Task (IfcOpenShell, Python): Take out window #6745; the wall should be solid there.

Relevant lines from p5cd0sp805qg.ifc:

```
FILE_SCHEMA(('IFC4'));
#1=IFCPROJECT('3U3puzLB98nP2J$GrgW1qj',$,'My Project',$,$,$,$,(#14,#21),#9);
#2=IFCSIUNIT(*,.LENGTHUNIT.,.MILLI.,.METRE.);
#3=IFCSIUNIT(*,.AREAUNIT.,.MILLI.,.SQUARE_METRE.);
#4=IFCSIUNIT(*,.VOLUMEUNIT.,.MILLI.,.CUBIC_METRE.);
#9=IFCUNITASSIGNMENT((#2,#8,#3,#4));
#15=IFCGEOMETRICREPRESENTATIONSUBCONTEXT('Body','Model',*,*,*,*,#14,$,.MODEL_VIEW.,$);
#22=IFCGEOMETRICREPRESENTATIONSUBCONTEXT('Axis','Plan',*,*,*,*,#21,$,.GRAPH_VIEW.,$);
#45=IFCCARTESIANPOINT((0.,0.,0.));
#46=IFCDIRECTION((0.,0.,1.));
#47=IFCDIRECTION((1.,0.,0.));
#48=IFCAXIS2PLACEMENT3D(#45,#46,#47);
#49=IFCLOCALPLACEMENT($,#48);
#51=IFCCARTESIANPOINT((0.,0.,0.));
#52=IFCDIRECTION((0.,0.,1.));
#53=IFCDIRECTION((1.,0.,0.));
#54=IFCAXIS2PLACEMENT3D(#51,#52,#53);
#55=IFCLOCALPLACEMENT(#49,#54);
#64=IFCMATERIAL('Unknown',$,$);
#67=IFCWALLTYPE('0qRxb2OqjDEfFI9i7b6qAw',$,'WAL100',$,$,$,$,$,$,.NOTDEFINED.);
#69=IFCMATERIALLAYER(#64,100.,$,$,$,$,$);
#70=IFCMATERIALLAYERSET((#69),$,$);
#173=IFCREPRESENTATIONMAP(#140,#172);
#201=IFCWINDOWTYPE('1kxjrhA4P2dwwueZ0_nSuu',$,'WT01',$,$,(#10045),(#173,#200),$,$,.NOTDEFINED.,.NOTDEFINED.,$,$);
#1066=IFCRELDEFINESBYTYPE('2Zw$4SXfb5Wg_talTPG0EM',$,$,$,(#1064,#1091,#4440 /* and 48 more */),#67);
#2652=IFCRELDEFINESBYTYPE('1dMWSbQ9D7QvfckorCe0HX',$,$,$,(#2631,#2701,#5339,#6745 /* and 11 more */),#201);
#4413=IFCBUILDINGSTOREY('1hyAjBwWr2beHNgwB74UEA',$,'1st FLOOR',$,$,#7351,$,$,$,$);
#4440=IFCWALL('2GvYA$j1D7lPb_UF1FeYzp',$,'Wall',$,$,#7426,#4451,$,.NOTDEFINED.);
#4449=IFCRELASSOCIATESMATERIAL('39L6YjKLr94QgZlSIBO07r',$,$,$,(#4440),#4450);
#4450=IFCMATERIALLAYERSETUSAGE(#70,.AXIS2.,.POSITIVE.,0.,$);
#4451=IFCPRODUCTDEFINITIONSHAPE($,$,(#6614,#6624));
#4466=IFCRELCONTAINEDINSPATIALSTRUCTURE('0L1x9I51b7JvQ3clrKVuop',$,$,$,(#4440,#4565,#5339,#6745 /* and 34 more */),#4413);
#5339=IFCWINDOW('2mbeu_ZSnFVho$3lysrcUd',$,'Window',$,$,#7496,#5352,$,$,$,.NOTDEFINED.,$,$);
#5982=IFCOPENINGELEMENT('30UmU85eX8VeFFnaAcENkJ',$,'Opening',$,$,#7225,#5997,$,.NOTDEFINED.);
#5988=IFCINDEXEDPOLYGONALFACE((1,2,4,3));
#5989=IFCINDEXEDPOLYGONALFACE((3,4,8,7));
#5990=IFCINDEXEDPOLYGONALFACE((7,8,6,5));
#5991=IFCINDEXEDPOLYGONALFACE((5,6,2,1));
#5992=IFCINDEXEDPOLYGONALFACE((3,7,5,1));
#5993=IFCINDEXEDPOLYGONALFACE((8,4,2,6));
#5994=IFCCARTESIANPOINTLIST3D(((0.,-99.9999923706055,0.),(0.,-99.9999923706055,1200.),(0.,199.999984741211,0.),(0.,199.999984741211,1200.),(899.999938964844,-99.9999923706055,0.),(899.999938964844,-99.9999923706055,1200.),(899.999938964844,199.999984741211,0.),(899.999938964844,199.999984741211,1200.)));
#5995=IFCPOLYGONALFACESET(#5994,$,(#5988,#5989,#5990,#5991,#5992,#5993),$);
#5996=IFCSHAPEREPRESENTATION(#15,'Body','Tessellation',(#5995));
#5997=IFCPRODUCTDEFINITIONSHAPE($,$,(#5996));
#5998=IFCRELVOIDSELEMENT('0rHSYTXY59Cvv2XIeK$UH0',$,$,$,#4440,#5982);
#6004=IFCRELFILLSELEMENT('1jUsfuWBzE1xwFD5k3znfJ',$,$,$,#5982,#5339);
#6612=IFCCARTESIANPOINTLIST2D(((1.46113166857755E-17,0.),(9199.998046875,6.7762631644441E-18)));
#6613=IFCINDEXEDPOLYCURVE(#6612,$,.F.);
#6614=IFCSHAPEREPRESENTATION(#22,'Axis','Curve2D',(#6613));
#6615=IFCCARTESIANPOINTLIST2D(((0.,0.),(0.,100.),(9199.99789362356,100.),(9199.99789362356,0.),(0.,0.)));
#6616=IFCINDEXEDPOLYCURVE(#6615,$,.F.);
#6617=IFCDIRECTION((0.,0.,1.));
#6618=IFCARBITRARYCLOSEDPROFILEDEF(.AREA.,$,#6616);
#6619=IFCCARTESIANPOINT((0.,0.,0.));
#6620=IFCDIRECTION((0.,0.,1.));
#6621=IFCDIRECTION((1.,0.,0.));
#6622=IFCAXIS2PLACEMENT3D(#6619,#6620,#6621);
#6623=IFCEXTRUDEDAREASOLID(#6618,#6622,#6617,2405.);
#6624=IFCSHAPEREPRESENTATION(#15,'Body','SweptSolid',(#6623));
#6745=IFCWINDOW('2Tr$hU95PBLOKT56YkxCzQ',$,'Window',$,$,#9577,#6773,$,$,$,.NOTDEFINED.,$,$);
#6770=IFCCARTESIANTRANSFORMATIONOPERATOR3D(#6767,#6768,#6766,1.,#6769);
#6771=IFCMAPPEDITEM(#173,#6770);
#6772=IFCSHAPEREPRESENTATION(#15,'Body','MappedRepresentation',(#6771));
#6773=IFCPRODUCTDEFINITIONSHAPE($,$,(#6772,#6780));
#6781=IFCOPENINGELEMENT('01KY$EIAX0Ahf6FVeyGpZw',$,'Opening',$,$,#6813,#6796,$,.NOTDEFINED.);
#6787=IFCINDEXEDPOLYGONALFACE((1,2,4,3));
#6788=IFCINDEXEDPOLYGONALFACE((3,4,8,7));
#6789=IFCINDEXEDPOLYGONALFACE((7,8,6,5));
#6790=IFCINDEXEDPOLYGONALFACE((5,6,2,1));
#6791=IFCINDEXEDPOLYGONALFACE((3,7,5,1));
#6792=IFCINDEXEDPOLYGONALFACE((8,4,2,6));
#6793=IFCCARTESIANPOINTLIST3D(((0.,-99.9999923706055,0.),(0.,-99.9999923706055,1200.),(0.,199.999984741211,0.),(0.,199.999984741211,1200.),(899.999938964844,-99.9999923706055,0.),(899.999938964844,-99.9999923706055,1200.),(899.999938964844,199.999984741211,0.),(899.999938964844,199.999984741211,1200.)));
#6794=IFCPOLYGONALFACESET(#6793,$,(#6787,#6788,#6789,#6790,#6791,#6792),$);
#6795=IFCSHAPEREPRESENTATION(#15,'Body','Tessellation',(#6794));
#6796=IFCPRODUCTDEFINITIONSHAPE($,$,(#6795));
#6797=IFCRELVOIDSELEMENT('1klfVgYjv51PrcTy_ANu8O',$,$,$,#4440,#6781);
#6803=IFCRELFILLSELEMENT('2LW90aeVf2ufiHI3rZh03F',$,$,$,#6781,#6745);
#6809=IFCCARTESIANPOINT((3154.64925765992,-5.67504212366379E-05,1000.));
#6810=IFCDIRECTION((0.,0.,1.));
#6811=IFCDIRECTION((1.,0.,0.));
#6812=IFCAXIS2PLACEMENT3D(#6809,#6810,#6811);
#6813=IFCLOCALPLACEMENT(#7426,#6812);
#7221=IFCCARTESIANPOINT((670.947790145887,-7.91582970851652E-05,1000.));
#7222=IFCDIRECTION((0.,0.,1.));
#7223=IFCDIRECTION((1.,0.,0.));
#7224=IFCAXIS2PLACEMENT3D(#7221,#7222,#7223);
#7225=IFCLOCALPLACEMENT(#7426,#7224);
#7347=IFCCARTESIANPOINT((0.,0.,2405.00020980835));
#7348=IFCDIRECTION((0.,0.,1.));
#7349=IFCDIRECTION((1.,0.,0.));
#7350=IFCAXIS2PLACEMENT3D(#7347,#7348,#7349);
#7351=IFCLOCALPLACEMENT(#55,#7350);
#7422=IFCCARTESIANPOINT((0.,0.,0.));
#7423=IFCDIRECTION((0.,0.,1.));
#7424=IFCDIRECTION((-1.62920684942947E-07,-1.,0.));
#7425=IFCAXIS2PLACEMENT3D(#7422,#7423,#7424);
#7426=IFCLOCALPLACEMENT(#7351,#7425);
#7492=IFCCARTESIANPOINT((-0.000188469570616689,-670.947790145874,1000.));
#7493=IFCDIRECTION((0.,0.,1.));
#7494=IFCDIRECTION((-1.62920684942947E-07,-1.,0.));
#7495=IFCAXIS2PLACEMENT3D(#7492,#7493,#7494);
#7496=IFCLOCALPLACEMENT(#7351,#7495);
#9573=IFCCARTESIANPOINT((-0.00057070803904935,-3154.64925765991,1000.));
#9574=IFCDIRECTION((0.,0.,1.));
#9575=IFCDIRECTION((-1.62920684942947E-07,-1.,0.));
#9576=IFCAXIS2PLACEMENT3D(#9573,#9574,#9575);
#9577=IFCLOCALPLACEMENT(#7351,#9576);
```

```python
import ifcopenshell
import ifcopenshell.api.feature
import ifcopenshell.api.root
import ifcopenshell.geom
import ifcopenshell.util.shape

model = ifcopenshell.open("p5cd0sp805qg.ifc")
settings = ifcopenshell.geom.settings()


def volume(element):
    """Net volume in cubic metres, openings subtracted."""
    shape = ifcopenshell.geom.create_shape(settings, element)
    return ifcopenshell.util.shape.get_volume(shape.geometry)


window = model.by_guid("2Tr$hU95PBLOKT56YkxCzQ")
opening = window.FillsVoids[0].RelatingOpeningElement
wall = opening.VoidsElements[0].RelatingBuildingElement
before = volume(wall)

ifcopenshell.api.root.remove_product(model, product=window)
ifcopenshell.api.feature.remove_feature(model, feature=opening)

after = volume(wall)

print(f"wall volume {before:.3f} -> {after:.3f} m3")

model.write("p5cd0sp805qg-out.ifc")
```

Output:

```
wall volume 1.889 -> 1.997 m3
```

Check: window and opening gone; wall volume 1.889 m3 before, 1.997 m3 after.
